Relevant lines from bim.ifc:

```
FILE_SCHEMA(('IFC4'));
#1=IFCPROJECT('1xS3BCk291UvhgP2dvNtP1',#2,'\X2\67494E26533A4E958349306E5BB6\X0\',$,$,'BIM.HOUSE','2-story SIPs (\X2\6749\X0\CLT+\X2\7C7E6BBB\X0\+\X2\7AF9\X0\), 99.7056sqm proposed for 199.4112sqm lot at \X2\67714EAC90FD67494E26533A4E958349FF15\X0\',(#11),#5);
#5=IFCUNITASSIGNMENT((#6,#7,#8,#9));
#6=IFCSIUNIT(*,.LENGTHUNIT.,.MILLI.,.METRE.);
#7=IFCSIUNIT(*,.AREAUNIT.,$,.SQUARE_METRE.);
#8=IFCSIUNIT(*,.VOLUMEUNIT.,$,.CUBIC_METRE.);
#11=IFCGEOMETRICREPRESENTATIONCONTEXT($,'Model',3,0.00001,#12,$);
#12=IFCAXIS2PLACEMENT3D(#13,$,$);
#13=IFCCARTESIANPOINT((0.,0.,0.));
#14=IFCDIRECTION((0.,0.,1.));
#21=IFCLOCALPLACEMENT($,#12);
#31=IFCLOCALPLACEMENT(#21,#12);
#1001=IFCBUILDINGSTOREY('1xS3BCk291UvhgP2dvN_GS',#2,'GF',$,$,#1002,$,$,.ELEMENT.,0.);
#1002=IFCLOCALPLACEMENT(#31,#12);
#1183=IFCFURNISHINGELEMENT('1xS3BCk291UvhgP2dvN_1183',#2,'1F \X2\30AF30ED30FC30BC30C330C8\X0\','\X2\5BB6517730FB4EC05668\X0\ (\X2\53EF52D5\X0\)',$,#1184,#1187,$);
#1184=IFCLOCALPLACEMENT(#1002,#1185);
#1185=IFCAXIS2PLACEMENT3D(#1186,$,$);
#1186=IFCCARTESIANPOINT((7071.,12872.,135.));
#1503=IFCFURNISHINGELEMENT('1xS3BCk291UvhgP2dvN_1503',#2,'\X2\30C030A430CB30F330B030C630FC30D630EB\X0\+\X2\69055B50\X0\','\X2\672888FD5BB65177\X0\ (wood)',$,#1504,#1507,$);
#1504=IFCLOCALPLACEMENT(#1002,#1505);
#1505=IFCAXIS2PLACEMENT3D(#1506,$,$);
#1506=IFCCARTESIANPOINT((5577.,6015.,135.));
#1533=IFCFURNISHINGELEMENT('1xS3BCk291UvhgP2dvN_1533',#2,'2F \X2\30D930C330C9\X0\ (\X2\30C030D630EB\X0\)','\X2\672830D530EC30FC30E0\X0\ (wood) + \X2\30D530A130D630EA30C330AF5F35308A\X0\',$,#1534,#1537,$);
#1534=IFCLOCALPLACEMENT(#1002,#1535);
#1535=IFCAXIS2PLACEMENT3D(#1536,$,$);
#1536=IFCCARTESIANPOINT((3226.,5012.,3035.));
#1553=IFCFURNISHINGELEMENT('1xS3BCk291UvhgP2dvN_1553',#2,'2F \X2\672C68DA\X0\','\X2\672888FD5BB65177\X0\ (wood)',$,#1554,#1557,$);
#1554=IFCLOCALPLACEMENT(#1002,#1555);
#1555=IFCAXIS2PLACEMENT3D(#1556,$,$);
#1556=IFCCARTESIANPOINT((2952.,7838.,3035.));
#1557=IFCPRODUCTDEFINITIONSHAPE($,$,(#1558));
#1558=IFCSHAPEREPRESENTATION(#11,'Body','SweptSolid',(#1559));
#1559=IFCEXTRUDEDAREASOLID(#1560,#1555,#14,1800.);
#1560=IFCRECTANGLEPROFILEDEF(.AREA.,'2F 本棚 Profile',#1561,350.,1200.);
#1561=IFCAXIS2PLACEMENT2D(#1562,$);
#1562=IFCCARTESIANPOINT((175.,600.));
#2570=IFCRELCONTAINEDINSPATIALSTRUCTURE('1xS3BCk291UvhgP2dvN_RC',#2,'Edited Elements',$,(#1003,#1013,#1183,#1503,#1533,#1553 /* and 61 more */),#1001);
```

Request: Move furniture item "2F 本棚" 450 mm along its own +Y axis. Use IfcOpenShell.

```python
import ifcopenshell
import ifcopenshell.api.geometry
import ifcopenshell.util.placement
import ifcopenshell.util.unit

model = ifcopenshell.open("bim.ifc")
unit_scale = ifcopenshell.util.unit.calculate_unit_scale(model)

item = model.by_guid("1xS3BCk291UvhgP2dvN_1553")
matrix = ifcopenshell.util.placement.get_local_placement(item.ObjectPlacement)
matrix[:3, 3] += matrix[:3, 1] * 0.45 / unit_scale
ifcopenshell.api.geometry.edit_object_placement(model, product=item, matrix=matrix, is_si=False)

print(ifcopenshell.util.placement.get_local_placement(item.ObjectPlacement).round(3) + 0.0)

model.write("bim_rev.ifc")
```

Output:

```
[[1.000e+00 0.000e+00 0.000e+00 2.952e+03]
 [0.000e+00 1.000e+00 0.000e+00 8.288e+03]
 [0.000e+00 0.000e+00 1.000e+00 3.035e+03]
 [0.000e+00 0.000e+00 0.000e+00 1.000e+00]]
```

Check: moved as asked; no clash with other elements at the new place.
